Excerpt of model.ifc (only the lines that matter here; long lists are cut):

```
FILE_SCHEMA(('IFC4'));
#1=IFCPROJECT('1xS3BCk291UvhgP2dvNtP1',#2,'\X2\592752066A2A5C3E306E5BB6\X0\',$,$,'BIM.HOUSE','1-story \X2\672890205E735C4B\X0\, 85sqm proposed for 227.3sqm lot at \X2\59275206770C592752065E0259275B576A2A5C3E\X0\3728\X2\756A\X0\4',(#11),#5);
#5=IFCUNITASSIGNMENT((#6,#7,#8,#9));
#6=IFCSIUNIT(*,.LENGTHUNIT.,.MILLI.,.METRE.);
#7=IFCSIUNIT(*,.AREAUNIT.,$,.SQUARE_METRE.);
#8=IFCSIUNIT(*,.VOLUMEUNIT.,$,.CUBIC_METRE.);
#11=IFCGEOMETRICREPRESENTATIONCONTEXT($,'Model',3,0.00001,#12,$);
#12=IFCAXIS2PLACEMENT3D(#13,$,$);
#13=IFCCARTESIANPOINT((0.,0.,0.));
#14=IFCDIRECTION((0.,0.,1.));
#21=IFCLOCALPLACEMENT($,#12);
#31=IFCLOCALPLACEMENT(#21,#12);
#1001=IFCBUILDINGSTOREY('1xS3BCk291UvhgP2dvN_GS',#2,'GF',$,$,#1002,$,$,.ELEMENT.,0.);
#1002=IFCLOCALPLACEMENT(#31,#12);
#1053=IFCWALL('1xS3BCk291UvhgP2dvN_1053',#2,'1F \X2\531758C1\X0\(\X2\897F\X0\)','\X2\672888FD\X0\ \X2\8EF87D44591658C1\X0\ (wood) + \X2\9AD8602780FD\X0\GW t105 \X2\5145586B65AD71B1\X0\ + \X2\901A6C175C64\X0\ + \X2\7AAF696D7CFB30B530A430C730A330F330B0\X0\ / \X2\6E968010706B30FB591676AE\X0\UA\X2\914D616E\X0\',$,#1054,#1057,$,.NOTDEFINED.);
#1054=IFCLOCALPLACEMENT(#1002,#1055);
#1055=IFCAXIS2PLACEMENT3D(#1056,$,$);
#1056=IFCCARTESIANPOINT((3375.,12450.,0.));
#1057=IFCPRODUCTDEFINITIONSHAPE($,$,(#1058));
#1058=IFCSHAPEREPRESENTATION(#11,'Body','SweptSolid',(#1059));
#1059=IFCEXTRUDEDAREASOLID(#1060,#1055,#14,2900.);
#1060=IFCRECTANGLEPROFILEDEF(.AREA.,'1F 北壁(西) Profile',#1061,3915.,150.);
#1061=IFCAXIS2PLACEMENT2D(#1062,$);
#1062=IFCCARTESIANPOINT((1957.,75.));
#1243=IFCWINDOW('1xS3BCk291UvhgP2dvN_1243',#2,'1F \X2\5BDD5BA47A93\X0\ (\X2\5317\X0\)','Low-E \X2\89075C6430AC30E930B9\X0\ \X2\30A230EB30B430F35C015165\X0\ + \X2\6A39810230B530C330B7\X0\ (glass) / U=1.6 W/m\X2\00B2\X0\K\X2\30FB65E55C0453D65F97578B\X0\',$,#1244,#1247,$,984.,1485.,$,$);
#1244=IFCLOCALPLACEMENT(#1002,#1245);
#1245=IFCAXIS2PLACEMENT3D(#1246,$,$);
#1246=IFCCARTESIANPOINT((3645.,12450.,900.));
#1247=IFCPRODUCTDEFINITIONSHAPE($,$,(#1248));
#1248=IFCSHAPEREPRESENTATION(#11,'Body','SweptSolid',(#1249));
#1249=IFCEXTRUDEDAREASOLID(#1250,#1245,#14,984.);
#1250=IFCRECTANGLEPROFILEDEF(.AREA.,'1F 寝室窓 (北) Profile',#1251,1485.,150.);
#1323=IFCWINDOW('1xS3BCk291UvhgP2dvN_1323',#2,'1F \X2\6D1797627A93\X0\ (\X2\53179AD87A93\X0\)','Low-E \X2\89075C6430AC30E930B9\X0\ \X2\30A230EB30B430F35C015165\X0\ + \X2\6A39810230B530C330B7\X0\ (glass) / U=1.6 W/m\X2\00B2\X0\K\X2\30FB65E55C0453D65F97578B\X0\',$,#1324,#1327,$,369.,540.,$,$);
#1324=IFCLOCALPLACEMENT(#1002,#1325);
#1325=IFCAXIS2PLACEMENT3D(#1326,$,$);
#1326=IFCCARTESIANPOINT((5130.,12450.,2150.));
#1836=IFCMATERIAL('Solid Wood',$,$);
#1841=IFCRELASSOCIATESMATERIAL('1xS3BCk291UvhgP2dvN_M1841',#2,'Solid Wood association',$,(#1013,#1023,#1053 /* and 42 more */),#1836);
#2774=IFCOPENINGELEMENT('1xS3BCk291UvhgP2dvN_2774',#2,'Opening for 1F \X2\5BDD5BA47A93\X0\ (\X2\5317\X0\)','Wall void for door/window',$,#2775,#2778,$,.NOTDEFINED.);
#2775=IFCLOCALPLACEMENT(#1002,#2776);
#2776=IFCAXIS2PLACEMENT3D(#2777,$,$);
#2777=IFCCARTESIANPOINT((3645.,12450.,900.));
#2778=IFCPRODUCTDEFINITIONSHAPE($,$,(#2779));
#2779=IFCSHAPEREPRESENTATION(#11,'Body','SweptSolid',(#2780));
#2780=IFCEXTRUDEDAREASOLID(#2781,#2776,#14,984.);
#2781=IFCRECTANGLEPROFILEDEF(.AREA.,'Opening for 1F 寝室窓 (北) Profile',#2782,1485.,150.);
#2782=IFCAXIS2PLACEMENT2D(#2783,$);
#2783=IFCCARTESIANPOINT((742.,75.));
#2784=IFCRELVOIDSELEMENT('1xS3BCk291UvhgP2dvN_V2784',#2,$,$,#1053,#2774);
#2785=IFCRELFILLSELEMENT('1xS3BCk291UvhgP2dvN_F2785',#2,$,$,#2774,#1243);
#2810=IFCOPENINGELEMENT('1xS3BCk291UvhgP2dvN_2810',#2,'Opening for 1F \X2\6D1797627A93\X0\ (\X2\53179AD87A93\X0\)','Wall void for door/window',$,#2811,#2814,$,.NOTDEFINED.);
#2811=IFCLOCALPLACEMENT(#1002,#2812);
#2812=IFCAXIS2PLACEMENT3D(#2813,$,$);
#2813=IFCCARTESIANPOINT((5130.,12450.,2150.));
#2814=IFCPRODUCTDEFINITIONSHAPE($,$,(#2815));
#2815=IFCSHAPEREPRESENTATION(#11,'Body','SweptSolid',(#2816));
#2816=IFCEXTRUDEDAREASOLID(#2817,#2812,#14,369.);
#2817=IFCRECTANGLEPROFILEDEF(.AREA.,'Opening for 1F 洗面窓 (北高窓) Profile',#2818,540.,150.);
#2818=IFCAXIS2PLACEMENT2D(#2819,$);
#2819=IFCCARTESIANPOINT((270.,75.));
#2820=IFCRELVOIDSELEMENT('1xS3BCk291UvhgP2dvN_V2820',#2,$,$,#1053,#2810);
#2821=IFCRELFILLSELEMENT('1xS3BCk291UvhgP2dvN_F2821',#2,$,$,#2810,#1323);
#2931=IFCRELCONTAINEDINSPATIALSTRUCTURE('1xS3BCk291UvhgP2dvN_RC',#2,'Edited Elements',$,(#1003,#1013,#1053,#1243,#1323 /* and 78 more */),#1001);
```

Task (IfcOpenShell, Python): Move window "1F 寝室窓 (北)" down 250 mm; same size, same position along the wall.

```python
import numpy as np
import ifcopenshell
import ifcopenshell.api.geometry
import ifcopenshell.util.placement
import ifcopenshell.util.unit

model = ifcopenshell.open("model.ifc")
unit_scale = ifcopenshell.util.unit.calculate_unit_scale(model)

window = model.by_guid("1xS3BCk291UvhgP2dvN_1243")
opening = window.FillsVoids[0].RelatingOpeningElement
dz = -0.25 / unit_scale

shift = np.array([0.0, 0.0, dz])
# The window is not placed relative to its opening, so move both.
for product in (opening, window):
    matrix = ifcopenshell.util.placement.get_local_placement(product.ObjectPlacement)
    matrix[:3, 3] += shift
    ifcopenshell.api.geometry.edit_object_placement(model, product=product, matrix=matrix, is_si=False)

print(f"moved by {dz * unit_scale:+.3f} m")

model.write("model-out.ifc")
```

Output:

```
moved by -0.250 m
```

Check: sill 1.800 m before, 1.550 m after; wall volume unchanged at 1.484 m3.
